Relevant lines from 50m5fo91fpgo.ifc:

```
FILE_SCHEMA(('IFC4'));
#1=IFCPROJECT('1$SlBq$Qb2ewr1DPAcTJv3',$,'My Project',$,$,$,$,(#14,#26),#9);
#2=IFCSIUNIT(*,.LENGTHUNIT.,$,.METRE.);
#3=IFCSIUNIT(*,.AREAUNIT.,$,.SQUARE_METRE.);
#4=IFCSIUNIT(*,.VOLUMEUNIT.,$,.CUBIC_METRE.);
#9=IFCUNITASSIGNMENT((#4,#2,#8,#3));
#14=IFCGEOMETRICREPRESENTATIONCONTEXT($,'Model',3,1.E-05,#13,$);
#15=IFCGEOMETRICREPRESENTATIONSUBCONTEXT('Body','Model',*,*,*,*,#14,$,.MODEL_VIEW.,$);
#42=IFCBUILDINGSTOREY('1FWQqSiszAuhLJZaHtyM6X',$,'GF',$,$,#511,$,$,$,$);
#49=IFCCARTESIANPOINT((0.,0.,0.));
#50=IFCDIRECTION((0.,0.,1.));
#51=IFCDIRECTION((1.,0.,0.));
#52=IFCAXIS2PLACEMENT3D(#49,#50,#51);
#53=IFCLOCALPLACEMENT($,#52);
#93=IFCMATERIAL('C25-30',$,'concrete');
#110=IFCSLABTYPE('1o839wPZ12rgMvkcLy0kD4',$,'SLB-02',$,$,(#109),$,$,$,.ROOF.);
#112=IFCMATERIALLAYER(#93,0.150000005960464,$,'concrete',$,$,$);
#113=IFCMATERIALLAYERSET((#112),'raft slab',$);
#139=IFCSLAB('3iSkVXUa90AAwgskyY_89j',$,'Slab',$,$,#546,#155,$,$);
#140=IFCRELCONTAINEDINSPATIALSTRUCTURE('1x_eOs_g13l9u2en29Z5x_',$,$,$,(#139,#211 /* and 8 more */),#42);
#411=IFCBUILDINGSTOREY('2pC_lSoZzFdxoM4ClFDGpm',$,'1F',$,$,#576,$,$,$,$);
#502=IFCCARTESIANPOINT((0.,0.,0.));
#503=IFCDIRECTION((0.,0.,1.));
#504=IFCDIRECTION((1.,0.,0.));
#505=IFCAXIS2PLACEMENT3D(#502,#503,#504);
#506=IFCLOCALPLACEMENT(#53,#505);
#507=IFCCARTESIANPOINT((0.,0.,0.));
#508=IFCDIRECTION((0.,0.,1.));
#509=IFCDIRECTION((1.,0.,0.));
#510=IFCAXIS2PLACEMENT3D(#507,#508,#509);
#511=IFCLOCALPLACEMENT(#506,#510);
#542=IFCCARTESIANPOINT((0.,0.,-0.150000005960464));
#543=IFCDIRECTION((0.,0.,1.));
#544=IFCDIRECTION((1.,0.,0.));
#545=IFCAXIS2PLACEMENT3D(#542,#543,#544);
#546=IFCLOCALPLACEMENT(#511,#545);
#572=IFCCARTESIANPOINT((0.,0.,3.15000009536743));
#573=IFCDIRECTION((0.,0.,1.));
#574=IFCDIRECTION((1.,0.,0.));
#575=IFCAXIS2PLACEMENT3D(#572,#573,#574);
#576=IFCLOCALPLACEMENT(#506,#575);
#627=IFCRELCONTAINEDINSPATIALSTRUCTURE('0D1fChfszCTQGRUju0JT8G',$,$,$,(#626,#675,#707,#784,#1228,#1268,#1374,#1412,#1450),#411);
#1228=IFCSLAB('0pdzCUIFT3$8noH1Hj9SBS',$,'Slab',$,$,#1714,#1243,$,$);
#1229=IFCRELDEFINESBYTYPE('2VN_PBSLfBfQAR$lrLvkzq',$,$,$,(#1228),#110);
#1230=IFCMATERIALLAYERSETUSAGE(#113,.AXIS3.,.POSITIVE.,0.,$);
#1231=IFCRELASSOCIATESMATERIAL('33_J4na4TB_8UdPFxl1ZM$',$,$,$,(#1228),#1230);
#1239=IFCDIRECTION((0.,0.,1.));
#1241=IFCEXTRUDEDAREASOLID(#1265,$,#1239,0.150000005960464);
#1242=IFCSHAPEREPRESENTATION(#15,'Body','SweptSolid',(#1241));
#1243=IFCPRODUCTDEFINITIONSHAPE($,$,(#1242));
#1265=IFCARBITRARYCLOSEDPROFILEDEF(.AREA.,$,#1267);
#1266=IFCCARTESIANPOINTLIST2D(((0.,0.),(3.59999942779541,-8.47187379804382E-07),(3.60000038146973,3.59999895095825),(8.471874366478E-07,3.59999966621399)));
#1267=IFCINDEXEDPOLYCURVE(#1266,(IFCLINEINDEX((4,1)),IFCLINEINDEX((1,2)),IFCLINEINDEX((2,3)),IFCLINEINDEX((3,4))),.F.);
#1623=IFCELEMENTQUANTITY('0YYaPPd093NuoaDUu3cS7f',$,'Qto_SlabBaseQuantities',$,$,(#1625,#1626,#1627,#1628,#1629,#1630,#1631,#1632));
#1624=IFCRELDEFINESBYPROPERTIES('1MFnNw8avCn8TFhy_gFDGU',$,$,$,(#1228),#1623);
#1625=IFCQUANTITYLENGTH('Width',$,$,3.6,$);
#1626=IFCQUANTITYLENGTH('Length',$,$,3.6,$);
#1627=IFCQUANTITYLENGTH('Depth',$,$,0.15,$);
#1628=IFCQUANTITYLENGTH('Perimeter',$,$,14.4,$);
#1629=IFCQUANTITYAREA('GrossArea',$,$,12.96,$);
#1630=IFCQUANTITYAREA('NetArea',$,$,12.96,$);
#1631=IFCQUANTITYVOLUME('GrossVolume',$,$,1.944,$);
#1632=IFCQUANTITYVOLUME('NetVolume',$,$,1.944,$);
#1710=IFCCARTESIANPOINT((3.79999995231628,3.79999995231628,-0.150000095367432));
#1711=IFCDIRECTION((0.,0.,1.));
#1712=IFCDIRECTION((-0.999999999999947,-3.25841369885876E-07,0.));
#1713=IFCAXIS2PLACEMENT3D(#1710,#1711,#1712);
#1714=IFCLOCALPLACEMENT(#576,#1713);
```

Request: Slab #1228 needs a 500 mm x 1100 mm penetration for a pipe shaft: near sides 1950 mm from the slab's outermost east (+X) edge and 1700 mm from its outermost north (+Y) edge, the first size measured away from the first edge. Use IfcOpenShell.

```python
import numpy as np
import ifcopenshell
import ifcopenshell.api.feature
import ifcopenshell.api.geometry
import ifcopenshell.api.pset
import ifcopenshell.api.root
import ifcopenshell.geom
import ifcopenshell.util.element
import ifcopenshell.util.placement
import ifcopenshell.util.representation
import ifcopenshell.util.shape
import ifcopenshell.util.unit

model = ifcopenshell.open("50m5fo91fpgo.ifc")
unit_scale = ifcopenshell.util.unit.calculate_unit_scale(model)
area_scale = ifcopenshell.util.unit.calculate_unit_scale(model, "AREAUNIT")
volume_scale = ifcopenshell.util.unit.calculate_unit_scale(model, "VOLUMEUNIT")
settings = ifcopenshell.geom.settings()


def volume(element):
    """Net volume in cubic metres, openings subtracted."""
    shape = ifcopenshell.geom.create_shape(settings, element)
    return ifcopenshell.util.shape.get_volume(shape.geometry)


slab = model.by_guid("0pdzCUIFT3$8noH1Hj9SBS")
before = volume(slab)

# Extent in the slab's own axes, in metres. The edges named are its -X and -Y sides.
slab_shape = ifcopenshell.geom.create_shape(settings, slab)
vertices = ifcopenshell.util.shape.get_vertices(slab_shape.geometry)
x_min, y_min, bottom = vertices.min(axis=0)
top = vertices[:, 2].max()

opening = ifcopenshell.api.root.create_entity(model, ifc_class="IfcOpeningElement", name="Pipe shaft opening", predefined_type="OPENING")
context = ifcopenshell.util.representation.get_context(model, "Model", "Body", "MODEL_VIEW")
width, depth = 0.5, 1.1
outline = [(0.0, 0.0), (width, 0.0), (width, depth), (0.0, depth), (0.0, 0.0)]
# Overshoot both faces by 50 mm so the cut is clean.
shape = ifcopenshell.api.geometry.add_slab_representation(
    model, context=context, depth=top - bottom + 0.1, polyline=outline
)
ifcopenshell.api.geometry.assign_representation(model, product=opening, representation=shape)

matrix = ifcopenshell.util.placement.get_local_placement(slab.ObjectPlacement)
matrix[:, 3] = matrix @ np.append(np.array([x_min + 1.95, y_min + 1.7, bottom - 0.05]) / unit_scale, 1.0)
ifcopenshell.api.geometry.edit_object_placement(model, product=opening, matrix=matrix, is_si=False)
ifcopenshell.api.feature.add_feature(model, feature=opening, element=slab)

after = volume(slab)

# Update the slab's stored quantities.
qto = model.by_id(ifcopenshell.util.element.get_pset(slab, "Qto_SlabBaseQuantities", should_inherit=False)["id"])
ifcopenshell.api.pset.edit_qto(model, qto=qto, properties={
    "NetArea": after / (top - bottom) / area_scale,
    "NetVolume": after / volume_scale,
})

print(f"slab volume {before:.3f} -> {after:.3f} m3")

model.write("50m5fo91fpgo-out.ifc")
```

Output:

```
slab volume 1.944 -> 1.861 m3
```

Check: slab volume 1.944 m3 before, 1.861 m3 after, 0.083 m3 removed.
